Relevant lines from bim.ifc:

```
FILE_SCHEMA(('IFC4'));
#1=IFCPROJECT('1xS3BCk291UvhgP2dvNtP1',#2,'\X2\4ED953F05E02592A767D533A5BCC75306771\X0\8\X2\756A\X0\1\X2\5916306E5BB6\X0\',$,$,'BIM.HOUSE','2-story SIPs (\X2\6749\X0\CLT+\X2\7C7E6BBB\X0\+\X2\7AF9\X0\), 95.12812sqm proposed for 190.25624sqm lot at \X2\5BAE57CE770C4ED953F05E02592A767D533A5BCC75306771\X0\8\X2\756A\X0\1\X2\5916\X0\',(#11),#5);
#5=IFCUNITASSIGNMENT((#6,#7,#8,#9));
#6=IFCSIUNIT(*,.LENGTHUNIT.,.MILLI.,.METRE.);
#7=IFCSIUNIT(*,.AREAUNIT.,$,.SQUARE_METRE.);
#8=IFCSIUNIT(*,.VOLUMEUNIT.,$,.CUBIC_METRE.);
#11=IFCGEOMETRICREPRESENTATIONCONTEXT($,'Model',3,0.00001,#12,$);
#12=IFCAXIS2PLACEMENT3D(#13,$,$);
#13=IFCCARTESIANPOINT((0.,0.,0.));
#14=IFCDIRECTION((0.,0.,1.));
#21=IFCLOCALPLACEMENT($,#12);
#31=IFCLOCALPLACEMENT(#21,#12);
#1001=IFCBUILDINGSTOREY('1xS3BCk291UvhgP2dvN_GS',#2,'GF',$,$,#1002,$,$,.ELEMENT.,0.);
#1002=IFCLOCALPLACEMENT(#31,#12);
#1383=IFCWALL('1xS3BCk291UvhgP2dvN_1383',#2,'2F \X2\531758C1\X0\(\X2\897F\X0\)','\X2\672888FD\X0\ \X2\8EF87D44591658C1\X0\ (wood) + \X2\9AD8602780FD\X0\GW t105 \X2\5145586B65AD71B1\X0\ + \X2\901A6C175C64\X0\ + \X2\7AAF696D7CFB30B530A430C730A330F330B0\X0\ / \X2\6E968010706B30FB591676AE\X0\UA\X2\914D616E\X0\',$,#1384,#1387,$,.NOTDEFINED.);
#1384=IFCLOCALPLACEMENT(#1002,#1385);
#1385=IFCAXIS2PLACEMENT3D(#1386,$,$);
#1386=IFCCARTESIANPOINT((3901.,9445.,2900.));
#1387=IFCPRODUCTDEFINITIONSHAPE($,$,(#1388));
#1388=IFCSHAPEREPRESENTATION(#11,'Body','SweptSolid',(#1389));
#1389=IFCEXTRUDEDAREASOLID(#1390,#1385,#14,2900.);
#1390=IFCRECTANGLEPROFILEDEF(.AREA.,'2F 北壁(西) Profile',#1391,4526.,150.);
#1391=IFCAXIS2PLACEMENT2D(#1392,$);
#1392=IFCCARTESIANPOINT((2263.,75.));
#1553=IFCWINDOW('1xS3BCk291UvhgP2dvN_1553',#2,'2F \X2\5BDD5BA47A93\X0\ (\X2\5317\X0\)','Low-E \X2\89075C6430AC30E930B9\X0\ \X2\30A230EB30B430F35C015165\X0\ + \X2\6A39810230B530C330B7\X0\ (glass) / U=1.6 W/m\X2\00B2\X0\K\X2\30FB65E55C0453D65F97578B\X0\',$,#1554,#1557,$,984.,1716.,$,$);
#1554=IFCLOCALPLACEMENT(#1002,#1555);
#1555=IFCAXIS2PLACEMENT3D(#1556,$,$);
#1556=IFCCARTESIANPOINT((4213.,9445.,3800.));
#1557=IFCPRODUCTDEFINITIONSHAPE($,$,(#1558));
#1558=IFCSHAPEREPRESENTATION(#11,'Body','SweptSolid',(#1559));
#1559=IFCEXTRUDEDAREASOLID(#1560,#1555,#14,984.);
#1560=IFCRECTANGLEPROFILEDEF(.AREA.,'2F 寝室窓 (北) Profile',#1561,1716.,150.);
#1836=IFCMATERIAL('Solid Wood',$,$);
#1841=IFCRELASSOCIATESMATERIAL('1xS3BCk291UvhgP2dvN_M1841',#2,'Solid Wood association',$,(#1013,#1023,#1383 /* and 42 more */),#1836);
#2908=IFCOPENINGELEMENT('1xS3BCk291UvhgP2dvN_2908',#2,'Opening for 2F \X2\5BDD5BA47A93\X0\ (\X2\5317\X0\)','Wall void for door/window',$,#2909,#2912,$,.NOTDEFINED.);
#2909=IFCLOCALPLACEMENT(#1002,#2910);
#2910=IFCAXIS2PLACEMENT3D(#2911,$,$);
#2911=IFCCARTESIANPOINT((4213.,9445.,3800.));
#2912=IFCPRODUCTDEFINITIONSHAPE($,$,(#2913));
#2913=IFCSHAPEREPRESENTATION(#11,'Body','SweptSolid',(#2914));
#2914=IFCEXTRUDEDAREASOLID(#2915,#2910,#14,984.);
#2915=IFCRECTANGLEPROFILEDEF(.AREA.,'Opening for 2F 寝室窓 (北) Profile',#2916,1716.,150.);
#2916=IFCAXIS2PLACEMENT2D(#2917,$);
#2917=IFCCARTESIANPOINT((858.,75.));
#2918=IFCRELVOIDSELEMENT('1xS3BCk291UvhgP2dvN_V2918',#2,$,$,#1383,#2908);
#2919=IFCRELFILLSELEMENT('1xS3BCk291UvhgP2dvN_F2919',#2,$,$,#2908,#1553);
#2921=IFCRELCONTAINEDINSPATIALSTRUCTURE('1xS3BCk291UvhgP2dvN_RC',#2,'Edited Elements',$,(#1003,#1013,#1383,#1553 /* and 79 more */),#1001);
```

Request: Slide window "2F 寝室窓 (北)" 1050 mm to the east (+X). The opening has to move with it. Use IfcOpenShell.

```python
import ifcopenshell
import ifcopenshell.api.geometry
import ifcopenshell.util.placement
import ifcopenshell.util.unit

model = ifcopenshell.open("bim.ifc")
unit_scale = ifcopenshell.util.unit.calculate_unit_scale(model)

window = model.by_guid("1xS3BCk291UvhgP2dvN_1553")
opening = window.FillsVoids[0].RelatingOpeningElement
wall = opening.VoidsElements[0].RelatingBuildingElement

wall_matrix = ifcopenshell.util.placement.get_local_placement(wall.ObjectPlacement)
shift = wall_matrix[:3, 0] * 1.05 / unit_scale
before = ifcopenshell.util.placement.get_local_placement(window.ObjectPlacement)[:3, 3].copy()

# The window is not placed relative to its opening, so move both.
for product in (opening, window):
    matrix = ifcopenshell.util.placement.get_local_placement(product.ObjectPlacement)
    matrix[:3, 3] += shift
    ifcopenshell.api.geometry.edit_object_placement(model, product=product, matrix=matrix, is_si=False)

after = ifcopenshell.util.placement.get_local_placement(window.ObjectPlacement)[:3, 3]
print("window moved by", (after - before).round(3) + 0.0)

model.write("bim_updated.ifc")
```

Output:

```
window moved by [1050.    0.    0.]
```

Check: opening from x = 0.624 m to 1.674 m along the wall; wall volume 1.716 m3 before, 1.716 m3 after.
